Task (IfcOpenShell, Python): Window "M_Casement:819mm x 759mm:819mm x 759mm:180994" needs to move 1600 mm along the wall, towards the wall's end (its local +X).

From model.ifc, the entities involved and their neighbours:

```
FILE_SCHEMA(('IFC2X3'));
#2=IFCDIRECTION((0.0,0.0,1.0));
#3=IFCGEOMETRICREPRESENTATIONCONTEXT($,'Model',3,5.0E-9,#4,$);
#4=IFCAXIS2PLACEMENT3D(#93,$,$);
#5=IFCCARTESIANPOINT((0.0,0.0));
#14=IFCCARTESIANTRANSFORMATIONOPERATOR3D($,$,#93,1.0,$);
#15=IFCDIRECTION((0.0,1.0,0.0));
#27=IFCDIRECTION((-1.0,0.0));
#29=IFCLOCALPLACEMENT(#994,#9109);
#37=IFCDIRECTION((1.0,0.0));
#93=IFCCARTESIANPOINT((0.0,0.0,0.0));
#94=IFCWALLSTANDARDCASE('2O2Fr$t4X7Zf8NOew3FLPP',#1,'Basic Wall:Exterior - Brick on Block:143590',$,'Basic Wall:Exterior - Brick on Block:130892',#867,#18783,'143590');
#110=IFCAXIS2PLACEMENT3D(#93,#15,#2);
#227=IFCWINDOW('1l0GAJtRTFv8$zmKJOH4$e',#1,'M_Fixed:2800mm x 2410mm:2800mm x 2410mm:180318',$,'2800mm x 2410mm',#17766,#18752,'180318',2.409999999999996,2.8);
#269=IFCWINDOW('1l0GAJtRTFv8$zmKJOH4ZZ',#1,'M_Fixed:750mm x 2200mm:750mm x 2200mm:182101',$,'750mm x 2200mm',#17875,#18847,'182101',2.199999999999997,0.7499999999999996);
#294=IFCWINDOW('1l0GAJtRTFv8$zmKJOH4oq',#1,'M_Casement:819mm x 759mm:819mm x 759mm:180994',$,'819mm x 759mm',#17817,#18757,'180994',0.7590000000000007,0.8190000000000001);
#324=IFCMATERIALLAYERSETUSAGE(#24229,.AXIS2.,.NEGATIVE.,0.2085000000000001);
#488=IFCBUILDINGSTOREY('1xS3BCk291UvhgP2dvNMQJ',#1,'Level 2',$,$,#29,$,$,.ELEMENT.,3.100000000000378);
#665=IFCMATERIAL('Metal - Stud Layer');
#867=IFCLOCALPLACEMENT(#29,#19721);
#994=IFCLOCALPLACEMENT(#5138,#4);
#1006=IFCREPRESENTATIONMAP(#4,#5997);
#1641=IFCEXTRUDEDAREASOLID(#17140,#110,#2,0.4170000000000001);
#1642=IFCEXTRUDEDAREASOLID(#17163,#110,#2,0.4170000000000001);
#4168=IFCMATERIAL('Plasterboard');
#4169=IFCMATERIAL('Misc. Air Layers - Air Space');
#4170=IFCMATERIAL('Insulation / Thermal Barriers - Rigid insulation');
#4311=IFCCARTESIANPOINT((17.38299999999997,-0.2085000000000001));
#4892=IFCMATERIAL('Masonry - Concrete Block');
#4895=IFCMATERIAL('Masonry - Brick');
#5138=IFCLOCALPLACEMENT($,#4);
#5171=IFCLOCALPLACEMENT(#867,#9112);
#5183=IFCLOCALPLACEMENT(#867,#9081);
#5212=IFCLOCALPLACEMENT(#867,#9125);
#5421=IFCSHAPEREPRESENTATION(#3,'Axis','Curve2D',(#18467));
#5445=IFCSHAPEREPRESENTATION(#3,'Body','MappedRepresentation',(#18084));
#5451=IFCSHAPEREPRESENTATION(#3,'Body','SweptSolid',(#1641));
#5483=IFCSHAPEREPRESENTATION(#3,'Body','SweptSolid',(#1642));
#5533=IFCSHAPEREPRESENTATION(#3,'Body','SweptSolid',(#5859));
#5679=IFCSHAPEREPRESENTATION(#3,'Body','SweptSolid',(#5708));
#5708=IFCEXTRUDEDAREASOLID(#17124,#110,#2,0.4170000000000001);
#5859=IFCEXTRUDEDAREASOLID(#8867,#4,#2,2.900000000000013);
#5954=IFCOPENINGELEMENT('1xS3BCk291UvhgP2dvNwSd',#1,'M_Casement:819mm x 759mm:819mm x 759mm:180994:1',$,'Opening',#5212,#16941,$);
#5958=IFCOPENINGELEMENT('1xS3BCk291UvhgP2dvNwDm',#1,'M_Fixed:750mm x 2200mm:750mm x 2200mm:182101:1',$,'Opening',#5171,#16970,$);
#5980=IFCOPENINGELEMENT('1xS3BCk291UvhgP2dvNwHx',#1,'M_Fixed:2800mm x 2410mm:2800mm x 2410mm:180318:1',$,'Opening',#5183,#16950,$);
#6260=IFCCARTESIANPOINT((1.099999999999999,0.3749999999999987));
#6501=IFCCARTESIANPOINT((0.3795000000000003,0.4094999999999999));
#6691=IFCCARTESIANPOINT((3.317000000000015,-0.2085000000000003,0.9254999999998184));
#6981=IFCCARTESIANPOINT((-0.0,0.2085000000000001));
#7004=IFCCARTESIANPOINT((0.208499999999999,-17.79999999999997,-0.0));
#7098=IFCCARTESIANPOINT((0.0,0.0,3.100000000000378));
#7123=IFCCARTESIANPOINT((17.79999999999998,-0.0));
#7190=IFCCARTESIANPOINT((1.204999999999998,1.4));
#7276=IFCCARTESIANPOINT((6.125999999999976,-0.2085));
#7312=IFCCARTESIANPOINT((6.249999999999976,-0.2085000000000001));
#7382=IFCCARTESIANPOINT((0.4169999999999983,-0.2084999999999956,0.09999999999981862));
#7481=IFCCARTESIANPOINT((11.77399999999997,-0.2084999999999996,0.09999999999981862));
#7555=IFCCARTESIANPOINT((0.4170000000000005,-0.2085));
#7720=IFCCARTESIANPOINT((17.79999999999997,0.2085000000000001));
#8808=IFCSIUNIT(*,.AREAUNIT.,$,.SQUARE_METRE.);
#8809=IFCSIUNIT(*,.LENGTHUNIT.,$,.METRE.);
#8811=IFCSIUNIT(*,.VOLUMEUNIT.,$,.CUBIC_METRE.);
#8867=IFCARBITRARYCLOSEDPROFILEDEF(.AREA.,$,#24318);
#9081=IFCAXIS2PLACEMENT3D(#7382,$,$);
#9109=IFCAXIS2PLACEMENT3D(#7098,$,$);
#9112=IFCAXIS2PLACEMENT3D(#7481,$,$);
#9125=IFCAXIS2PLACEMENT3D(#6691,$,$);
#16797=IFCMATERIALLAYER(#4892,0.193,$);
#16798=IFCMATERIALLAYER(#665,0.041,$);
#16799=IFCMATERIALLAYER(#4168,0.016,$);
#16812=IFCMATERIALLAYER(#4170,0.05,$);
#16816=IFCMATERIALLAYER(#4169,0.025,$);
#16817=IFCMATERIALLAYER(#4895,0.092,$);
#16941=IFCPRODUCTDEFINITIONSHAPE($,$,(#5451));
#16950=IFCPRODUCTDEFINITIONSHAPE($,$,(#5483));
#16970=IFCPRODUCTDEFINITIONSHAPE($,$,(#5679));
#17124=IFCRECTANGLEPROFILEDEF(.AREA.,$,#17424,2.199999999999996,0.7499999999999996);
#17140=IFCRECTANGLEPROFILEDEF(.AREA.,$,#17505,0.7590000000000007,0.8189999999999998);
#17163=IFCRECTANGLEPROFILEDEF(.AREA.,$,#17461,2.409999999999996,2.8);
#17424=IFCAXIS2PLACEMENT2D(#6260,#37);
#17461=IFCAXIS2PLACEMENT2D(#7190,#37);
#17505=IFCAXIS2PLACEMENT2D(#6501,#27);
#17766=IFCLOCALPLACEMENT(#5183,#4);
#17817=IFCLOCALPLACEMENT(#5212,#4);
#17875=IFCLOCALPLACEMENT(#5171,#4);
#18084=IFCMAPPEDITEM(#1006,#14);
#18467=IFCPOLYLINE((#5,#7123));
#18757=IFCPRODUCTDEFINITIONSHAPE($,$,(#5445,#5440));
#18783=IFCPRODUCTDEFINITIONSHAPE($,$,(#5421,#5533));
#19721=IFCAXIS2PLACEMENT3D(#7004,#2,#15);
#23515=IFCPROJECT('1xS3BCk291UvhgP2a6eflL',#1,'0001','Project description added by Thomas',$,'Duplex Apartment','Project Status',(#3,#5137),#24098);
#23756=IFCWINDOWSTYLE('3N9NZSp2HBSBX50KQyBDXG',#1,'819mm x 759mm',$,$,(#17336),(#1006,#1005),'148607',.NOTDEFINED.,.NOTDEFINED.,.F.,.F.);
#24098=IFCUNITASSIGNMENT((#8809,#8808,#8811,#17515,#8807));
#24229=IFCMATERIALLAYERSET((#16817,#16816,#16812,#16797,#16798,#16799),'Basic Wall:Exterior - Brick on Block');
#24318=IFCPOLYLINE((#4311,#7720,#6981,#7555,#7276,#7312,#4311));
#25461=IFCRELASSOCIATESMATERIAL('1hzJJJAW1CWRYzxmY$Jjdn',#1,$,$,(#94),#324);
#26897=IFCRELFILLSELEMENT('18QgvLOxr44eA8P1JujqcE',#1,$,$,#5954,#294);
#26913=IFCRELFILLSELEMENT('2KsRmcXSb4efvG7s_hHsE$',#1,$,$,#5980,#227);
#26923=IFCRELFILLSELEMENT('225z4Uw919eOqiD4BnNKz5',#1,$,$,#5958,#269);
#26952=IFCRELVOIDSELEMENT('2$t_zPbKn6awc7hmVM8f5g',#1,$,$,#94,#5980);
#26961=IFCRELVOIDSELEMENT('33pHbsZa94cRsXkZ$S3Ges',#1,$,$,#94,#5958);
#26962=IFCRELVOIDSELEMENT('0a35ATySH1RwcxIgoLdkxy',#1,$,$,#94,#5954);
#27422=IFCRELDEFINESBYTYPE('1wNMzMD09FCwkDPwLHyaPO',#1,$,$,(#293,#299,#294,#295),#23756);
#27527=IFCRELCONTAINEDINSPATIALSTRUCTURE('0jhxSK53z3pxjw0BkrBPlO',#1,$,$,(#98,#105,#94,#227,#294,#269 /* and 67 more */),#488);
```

```python
import ifcopenshell
import ifcopenshell.api.geometry
import ifcopenshell.util.placement
import ifcopenshell.util.unit

model = ifcopenshell.open("model.ifc")
unit_scale = ifcopenshell.util.unit.calculate_unit_scale(model)

window = model.by_id(294)
opening = window.FillsVoids[0].RelatingOpeningElement
wall = opening.VoidsElements[0].RelatingBuildingElement

wall_matrix = ifcopenshell.util.placement.get_local_placement(wall.ObjectPlacement)
shift = wall_matrix[:3, 0] * 1.6 / unit_scale
before = ifcopenshell.util.placement.get_local_placement(window.ObjectPlacement)[:3, 3].copy()

# The window is placed relative to its opening, so it follows when the opening moves.
matrix = ifcopenshell.util.placement.get_local_placement(opening.ObjectPlacement)
matrix[:3, 3] += shift
ifcopenshell.api.geometry.edit_object_placement(
    model, product=opening, matrix=matrix, is_si=False, should_transform_children=True
)

after = ifcopenshell.util.placement.get_local_placement(window.ObjectPlacement)[:3, 3]
print("window moved by", (after - before).round(3) + 0.0)

model.write("model_edited.ifc")
```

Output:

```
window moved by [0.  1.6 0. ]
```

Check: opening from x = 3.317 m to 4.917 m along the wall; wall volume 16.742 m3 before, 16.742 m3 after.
